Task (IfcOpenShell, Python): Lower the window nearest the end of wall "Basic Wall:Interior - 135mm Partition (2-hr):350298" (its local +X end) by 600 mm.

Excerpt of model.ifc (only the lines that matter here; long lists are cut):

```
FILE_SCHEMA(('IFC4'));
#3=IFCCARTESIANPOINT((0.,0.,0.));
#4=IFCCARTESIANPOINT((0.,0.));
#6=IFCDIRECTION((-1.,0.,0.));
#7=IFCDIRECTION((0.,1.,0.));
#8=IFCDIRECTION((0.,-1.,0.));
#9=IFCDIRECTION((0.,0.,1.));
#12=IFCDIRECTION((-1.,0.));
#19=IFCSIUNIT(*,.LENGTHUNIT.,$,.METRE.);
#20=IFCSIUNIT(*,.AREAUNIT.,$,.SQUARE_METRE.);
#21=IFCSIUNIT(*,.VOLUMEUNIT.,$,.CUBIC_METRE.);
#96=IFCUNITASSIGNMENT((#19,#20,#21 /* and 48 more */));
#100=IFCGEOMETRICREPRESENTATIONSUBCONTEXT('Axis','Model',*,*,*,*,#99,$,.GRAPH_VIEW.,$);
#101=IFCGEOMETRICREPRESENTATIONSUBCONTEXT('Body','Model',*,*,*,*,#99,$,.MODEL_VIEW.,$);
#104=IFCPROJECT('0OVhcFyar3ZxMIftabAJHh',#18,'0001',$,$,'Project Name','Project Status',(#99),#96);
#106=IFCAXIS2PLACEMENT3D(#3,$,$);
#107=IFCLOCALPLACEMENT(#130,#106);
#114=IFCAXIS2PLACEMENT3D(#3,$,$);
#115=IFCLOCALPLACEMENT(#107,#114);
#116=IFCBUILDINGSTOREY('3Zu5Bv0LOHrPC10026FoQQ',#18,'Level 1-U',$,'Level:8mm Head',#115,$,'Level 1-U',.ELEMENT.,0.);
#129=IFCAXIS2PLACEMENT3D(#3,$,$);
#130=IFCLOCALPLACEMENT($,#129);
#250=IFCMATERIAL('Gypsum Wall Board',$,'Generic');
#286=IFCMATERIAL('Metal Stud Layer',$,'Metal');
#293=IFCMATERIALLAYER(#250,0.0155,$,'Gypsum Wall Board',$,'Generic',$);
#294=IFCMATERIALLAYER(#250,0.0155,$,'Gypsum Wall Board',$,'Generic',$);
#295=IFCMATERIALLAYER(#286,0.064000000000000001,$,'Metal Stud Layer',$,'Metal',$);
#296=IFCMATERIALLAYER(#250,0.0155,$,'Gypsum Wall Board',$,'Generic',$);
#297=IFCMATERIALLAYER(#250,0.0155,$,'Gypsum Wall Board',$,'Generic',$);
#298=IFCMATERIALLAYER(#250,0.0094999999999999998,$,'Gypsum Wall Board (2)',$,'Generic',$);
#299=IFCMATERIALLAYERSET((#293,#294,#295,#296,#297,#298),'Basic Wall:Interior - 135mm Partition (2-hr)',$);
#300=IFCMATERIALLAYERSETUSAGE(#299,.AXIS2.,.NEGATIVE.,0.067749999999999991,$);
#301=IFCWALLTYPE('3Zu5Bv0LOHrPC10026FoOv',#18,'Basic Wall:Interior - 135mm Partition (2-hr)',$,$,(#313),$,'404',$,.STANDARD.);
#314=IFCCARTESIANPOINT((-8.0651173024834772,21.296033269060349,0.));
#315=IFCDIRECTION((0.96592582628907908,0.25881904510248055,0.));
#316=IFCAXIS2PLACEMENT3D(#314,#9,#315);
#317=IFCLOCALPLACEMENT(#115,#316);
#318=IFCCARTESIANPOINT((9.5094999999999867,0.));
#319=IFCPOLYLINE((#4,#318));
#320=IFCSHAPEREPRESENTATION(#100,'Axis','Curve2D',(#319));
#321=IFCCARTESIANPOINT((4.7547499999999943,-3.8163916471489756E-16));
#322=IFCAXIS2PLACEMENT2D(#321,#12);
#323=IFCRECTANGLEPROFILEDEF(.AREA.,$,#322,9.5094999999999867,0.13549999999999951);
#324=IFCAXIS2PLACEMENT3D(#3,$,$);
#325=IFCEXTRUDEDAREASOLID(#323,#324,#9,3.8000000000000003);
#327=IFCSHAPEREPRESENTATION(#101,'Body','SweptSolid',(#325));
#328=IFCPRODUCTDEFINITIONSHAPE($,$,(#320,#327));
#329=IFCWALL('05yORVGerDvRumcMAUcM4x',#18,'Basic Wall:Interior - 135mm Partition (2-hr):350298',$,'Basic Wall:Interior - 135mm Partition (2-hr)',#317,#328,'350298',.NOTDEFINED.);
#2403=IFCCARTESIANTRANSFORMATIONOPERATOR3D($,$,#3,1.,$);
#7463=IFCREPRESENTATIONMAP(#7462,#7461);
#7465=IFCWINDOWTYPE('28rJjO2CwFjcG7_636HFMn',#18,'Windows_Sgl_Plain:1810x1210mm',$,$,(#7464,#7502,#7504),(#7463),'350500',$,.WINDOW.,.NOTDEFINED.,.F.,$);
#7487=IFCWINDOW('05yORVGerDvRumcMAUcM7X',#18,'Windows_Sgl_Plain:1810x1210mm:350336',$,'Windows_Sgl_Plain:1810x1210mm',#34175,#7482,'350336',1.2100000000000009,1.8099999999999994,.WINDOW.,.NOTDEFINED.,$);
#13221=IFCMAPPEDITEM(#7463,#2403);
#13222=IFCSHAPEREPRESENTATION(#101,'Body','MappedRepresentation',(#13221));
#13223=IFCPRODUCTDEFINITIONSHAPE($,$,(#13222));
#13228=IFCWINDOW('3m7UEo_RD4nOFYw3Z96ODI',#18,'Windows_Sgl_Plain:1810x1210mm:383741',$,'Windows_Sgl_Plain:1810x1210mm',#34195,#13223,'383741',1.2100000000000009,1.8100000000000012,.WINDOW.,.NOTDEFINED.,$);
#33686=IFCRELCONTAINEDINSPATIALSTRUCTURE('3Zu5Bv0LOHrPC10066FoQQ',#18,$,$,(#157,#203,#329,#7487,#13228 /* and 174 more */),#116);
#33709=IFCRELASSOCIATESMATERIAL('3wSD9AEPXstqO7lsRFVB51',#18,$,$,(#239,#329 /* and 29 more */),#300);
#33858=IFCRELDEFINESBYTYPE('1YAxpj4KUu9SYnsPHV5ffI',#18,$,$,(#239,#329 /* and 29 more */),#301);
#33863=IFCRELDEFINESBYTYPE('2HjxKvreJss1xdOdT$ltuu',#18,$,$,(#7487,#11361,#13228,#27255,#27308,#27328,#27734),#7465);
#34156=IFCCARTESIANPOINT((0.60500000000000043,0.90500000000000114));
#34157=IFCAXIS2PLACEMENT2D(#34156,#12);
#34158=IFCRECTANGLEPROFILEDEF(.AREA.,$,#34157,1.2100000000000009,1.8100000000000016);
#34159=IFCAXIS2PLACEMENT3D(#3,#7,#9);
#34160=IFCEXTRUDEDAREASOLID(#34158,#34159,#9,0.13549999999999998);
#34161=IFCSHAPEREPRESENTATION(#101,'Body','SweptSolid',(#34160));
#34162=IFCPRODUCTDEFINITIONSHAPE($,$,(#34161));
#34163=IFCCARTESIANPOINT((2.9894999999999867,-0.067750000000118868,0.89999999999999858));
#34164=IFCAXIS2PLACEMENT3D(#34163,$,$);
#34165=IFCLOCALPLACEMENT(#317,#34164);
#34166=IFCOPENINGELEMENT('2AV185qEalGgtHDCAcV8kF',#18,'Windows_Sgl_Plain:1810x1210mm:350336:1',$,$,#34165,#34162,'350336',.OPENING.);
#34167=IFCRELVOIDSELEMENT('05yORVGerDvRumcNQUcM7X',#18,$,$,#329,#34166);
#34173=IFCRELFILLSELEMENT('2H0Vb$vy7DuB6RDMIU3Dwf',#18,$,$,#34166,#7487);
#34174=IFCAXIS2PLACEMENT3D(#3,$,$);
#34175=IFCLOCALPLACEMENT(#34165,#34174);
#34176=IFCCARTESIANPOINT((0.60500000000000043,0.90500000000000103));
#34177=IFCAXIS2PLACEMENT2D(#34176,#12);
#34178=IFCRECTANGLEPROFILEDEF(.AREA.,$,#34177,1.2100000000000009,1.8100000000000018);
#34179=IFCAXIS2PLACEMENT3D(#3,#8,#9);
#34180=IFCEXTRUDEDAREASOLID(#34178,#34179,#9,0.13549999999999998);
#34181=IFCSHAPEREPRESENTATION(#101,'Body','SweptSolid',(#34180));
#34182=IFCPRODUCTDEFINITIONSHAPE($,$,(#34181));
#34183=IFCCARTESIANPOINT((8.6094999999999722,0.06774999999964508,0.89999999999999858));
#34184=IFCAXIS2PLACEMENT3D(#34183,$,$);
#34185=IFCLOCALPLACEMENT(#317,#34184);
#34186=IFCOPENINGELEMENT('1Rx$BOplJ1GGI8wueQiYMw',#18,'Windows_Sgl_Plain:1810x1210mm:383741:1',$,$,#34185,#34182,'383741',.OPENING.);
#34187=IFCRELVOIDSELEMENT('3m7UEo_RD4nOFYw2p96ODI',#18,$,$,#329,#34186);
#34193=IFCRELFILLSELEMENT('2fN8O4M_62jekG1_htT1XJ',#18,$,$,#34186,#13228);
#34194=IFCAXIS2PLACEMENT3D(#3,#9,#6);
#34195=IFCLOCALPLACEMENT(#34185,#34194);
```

```python
import numpy as np
import ifcopenshell
import ifcopenshell.api.geometry
import ifcopenshell.util.placement
import ifcopenshell.util.unit

model = ifcopenshell.open("model.ifc")
unit_scale = ifcopenshell.util.unit.calculate_unit_scale(model)

window = model.by_id(13228)
opening = window.FillsVoids[0].RelatingOpeningElement
dz = -0.6 / unit_scale

shift = np.array([0.0, 0.0, dz])
# The window is placed relative to its opening, so it follows when the opening moves.
matrix = ifcopenshell.util.placement.get_local_placement(opening.ObjectPlacement)
matrix[:3, 3] += shift
ifcopenshell.api.geometry.edit_object_placement(
    model, product=opening, matrix=matrix, is_si=False, should_transform_children=True
)

print(f"moved by {dz * unit_scale:+.3f} m")

model.write("model_rev.ifc")
```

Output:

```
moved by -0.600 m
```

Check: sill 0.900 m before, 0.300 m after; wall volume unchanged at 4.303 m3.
